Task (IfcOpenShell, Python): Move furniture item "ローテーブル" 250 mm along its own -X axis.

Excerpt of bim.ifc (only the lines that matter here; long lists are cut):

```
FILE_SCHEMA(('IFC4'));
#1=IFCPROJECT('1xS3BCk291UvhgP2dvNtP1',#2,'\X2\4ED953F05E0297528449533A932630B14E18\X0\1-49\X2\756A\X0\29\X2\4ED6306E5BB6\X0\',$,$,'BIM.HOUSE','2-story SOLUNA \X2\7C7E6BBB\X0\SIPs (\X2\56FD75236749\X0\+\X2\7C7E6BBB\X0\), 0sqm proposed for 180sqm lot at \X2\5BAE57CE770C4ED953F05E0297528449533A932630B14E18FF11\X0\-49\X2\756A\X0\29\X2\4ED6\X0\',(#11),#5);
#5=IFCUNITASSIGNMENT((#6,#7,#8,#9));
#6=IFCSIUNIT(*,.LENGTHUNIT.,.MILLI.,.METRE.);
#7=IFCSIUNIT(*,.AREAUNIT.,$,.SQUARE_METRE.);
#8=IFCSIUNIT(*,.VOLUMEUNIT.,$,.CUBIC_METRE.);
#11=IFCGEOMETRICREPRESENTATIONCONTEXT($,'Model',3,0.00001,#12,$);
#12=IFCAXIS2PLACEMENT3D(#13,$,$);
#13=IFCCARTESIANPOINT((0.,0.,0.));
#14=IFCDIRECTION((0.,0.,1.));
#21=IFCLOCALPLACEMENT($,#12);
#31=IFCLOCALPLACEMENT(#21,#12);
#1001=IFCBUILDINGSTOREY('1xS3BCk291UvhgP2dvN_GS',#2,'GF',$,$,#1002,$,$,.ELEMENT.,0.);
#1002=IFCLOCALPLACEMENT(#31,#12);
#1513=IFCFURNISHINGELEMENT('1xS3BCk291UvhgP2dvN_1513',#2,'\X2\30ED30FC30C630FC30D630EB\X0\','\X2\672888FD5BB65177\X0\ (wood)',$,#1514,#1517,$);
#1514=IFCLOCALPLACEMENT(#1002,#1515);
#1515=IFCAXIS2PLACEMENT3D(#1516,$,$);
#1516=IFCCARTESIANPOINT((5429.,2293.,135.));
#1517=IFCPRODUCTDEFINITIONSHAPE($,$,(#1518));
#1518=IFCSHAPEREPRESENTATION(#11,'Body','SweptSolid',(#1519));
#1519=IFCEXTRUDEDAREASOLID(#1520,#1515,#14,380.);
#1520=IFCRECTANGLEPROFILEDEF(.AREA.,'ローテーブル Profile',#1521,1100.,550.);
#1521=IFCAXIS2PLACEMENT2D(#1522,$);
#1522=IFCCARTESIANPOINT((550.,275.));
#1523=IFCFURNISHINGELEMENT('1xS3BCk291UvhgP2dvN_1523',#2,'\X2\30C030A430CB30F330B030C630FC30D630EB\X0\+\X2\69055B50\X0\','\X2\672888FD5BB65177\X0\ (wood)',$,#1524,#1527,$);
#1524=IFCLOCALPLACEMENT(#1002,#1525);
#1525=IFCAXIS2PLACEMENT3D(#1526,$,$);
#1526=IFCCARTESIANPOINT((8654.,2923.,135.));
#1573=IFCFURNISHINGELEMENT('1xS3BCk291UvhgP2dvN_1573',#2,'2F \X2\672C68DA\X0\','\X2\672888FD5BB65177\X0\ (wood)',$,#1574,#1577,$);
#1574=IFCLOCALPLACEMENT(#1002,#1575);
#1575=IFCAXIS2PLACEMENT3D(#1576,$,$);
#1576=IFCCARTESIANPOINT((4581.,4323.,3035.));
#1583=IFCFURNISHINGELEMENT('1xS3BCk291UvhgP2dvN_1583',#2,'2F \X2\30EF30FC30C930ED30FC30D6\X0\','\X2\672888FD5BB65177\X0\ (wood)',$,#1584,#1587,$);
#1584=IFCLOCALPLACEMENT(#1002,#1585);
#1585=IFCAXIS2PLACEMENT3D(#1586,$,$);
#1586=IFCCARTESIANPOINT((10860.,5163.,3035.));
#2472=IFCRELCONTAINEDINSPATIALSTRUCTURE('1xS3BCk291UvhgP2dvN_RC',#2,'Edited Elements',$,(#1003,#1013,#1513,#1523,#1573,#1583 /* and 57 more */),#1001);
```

```python
import ifcopenshell
import ifcopenshell.api.geometry
import ifcopenshell.util.placement
import ifcopenshell.util.unit

model = ifcopenshell.open("bim.ifc")
unit_scale = ifcopenshell.util.unit.calculate_unit_scale(model)

item = model.by_guid("1xS3BCk291UvhgP2dvN_1513")
matrix = ifcopenshell.util.placement.get_local_placement(item.ObjectPlacement)
matrix[:3, 3] -= matrix[:3, 0] * 0.25 / unit_scale
ifcopenshell.api.geometry.edit_object_placement(model, product=item, matrix=matrix, is_si=False)

print(ifcopenshell.util.placement.get_local_placement(item.ObjectPlacement).round(3) + 0.0)

model.write("bim_v2.ifc")
```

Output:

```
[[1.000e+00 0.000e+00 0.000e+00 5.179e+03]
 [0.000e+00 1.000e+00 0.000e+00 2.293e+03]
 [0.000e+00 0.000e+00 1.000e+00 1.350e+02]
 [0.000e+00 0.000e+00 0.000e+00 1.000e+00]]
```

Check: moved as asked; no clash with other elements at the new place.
